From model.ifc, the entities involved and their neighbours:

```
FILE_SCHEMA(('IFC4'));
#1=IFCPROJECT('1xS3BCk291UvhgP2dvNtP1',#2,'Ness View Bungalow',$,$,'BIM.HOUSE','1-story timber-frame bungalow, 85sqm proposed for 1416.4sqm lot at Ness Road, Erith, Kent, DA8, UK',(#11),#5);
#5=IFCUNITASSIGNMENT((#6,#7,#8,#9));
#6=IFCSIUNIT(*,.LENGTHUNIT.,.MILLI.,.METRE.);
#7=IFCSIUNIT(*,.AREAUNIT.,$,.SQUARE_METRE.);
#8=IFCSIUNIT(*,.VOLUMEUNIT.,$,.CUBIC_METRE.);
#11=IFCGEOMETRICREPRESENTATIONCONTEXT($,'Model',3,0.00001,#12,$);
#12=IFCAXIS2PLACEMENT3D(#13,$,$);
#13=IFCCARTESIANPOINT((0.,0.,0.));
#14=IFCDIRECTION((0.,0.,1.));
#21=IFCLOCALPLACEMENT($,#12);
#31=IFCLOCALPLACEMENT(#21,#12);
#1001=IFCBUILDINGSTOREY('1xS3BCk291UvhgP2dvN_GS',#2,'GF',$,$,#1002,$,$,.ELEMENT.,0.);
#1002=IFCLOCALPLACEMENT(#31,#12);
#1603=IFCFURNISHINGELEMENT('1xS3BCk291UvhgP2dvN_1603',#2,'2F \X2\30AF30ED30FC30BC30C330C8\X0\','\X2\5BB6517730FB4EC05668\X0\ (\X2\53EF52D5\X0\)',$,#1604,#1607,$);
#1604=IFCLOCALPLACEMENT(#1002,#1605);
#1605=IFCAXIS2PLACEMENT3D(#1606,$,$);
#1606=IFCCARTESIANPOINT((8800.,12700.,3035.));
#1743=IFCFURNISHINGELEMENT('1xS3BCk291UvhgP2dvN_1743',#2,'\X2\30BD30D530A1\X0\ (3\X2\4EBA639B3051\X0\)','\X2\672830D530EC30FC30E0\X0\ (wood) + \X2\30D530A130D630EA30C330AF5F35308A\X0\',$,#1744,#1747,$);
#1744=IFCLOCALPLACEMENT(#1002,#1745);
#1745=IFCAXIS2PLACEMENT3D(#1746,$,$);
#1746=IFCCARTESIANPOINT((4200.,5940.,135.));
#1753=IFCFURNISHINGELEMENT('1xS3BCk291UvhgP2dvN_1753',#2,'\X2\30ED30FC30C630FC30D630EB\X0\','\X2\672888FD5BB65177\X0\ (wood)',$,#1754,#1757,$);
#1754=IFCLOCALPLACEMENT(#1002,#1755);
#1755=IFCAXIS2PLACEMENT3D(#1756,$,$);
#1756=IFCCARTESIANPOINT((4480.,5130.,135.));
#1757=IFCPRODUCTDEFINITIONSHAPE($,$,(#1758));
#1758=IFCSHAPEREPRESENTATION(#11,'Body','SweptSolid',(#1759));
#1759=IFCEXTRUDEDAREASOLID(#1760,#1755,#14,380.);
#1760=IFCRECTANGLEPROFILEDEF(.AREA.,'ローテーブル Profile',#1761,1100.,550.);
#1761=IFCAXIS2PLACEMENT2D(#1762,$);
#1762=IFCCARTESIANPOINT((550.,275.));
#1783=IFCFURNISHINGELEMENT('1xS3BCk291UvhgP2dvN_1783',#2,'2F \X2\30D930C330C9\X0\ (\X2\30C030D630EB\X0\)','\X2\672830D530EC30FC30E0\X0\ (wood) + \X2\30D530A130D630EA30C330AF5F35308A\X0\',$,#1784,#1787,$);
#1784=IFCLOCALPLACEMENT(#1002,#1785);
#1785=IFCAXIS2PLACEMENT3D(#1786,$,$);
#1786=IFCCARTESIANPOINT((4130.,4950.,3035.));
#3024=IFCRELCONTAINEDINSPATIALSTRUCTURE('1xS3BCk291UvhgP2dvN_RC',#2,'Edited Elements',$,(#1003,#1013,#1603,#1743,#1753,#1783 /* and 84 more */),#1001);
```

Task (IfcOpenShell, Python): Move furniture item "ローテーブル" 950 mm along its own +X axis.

```python
import ifcopenshell
import ifcopenshell.api.geometry
import ifcopenshell.util.placement
import ifcopenshell.util.unit

model = ifcopenshell.open("model.ifc")
unit_scale = ifcopenshell.util.unit.calculate_unit_scale(model)

item = model.by_guid("1xS3BCk291UvhgP2dvN_1753")
matrix = ifcopenshell.util.placement.get_local_placement(item.ObjectPlacement)
matrix[:3, 3] += matrix[:3, 0] * 0.95 / unit_scale
ifcopenshell.api.geometry.edit_object_placement(model, product=item, matrix=matrix, is_si=False)

print(ifcopenshell.util.placement.get_local_placement(item.ObjectPlacement).round(3) + 0.0)

model.write("model-out.ifc")
```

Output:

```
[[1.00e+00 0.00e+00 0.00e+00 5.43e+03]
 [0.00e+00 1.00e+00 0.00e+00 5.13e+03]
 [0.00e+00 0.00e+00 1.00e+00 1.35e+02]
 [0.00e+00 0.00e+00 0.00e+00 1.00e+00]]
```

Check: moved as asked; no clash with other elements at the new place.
